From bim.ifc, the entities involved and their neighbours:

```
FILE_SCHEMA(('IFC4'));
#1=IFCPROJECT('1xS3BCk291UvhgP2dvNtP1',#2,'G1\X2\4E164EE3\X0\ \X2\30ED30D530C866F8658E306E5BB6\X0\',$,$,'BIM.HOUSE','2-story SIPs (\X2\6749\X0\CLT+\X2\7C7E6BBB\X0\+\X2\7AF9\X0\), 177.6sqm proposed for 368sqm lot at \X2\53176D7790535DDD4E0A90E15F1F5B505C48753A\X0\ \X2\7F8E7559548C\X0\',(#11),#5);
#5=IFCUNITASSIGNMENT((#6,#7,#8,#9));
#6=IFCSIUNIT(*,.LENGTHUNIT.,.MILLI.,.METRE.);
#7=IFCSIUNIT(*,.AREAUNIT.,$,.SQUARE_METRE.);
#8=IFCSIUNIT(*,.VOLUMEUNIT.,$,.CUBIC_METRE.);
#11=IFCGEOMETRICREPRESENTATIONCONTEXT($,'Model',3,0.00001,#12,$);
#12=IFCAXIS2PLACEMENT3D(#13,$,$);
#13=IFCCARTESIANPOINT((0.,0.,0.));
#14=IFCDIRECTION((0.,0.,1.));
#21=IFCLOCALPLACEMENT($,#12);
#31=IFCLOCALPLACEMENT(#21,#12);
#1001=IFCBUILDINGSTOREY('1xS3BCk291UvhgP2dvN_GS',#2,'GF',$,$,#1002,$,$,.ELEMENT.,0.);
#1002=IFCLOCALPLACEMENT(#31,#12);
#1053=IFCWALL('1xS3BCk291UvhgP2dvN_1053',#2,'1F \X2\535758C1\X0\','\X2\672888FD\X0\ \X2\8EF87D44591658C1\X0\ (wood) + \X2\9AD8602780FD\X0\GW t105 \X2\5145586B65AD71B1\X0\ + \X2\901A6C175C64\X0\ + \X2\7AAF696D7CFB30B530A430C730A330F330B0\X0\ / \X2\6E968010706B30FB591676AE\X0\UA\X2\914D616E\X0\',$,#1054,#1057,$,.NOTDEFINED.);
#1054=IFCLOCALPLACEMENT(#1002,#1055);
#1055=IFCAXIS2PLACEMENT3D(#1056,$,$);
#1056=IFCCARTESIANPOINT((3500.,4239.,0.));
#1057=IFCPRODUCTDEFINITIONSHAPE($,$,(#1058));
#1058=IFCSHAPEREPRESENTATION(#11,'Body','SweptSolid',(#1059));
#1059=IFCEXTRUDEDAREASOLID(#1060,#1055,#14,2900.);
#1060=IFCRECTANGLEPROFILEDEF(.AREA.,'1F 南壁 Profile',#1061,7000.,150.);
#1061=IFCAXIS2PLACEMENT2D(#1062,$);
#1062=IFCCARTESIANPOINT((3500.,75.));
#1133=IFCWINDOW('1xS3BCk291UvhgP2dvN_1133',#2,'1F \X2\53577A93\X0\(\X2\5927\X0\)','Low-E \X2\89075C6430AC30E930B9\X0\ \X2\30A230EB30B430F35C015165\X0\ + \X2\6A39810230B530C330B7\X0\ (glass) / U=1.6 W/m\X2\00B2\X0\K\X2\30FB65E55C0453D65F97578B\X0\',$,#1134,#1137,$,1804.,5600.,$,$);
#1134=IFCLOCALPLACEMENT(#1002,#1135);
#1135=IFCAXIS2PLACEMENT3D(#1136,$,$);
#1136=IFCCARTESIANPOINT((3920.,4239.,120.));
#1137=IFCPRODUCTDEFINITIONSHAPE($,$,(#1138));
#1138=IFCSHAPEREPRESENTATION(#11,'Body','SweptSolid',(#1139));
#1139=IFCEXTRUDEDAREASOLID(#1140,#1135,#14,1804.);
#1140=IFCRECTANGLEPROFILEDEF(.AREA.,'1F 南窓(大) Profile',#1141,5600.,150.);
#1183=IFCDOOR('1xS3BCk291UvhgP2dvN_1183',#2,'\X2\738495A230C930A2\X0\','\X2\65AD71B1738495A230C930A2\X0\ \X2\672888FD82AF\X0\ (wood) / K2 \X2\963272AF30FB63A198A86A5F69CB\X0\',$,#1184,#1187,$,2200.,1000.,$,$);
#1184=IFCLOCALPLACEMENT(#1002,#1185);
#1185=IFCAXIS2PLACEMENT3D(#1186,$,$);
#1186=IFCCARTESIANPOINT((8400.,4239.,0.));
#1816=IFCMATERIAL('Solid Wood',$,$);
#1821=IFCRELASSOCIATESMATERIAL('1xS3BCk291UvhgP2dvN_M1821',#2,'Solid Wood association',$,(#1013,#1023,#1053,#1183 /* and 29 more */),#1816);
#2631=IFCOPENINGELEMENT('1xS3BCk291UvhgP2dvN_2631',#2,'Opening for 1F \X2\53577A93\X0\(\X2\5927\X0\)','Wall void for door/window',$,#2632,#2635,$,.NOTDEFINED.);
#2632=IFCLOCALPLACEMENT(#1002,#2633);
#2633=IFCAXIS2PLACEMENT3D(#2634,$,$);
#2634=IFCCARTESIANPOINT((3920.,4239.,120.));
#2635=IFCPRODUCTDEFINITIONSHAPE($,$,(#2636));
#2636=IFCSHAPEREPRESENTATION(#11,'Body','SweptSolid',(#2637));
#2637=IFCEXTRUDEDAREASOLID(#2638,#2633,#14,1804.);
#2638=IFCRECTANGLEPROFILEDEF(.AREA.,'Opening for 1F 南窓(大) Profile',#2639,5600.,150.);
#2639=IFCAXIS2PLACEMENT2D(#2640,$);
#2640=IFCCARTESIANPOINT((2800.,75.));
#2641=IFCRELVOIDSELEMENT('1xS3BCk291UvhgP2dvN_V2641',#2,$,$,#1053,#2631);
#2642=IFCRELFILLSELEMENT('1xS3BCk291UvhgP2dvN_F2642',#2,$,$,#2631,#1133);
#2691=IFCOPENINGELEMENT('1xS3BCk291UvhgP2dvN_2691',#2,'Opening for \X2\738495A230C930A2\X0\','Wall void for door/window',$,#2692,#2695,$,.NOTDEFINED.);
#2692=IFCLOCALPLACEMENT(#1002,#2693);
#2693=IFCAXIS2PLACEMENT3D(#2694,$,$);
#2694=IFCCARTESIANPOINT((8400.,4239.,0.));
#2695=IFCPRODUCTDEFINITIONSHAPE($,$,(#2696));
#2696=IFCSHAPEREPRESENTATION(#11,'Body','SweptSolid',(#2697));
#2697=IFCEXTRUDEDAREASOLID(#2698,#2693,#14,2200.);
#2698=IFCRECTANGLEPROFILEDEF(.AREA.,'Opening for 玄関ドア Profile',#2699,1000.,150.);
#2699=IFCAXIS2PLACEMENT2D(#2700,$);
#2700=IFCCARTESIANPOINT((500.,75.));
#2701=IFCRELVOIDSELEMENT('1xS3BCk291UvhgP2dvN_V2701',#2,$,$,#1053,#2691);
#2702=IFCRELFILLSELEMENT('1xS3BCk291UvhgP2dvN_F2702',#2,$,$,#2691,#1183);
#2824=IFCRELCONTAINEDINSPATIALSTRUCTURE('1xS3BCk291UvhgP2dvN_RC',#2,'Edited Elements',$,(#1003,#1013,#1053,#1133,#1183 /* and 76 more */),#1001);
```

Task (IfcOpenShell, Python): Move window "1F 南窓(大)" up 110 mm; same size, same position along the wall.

```python
import numpy as np
import ifcopenshell
import ifcopenshell.api.geometry
import ifcopenshell.util.placement
import ifcopenshell.util.unit

model = ifcopenshell.open("bim.ifc")
unit_scale = ifcopenshell.util.unit.calculate_unit_scale(model)

window = model.by_guid("1xS3BCk291UvhgP2dvN_1133")
opening = window.FillsVoids[0].RelatingOpeningElement
dz = 110.0

shift = np.array([0.0, 0.0, dz])
# The window is not placed relative to its opening, so move both.
for product in (opening, window):
    matrix = ifcopenshell.util.placement.get_local_placement(product.ObjectPlacement)
    matrix[:3, 3] += shift
    ifcopenshell.api.geometry.edit_object_placement(model, product=product, matrix=matrix, is_si=False)

print(f"moved by {dz * unit_scale:+.3f} m")

model.write("bim-out.ifc")
```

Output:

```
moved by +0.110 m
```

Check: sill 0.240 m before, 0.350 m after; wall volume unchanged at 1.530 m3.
